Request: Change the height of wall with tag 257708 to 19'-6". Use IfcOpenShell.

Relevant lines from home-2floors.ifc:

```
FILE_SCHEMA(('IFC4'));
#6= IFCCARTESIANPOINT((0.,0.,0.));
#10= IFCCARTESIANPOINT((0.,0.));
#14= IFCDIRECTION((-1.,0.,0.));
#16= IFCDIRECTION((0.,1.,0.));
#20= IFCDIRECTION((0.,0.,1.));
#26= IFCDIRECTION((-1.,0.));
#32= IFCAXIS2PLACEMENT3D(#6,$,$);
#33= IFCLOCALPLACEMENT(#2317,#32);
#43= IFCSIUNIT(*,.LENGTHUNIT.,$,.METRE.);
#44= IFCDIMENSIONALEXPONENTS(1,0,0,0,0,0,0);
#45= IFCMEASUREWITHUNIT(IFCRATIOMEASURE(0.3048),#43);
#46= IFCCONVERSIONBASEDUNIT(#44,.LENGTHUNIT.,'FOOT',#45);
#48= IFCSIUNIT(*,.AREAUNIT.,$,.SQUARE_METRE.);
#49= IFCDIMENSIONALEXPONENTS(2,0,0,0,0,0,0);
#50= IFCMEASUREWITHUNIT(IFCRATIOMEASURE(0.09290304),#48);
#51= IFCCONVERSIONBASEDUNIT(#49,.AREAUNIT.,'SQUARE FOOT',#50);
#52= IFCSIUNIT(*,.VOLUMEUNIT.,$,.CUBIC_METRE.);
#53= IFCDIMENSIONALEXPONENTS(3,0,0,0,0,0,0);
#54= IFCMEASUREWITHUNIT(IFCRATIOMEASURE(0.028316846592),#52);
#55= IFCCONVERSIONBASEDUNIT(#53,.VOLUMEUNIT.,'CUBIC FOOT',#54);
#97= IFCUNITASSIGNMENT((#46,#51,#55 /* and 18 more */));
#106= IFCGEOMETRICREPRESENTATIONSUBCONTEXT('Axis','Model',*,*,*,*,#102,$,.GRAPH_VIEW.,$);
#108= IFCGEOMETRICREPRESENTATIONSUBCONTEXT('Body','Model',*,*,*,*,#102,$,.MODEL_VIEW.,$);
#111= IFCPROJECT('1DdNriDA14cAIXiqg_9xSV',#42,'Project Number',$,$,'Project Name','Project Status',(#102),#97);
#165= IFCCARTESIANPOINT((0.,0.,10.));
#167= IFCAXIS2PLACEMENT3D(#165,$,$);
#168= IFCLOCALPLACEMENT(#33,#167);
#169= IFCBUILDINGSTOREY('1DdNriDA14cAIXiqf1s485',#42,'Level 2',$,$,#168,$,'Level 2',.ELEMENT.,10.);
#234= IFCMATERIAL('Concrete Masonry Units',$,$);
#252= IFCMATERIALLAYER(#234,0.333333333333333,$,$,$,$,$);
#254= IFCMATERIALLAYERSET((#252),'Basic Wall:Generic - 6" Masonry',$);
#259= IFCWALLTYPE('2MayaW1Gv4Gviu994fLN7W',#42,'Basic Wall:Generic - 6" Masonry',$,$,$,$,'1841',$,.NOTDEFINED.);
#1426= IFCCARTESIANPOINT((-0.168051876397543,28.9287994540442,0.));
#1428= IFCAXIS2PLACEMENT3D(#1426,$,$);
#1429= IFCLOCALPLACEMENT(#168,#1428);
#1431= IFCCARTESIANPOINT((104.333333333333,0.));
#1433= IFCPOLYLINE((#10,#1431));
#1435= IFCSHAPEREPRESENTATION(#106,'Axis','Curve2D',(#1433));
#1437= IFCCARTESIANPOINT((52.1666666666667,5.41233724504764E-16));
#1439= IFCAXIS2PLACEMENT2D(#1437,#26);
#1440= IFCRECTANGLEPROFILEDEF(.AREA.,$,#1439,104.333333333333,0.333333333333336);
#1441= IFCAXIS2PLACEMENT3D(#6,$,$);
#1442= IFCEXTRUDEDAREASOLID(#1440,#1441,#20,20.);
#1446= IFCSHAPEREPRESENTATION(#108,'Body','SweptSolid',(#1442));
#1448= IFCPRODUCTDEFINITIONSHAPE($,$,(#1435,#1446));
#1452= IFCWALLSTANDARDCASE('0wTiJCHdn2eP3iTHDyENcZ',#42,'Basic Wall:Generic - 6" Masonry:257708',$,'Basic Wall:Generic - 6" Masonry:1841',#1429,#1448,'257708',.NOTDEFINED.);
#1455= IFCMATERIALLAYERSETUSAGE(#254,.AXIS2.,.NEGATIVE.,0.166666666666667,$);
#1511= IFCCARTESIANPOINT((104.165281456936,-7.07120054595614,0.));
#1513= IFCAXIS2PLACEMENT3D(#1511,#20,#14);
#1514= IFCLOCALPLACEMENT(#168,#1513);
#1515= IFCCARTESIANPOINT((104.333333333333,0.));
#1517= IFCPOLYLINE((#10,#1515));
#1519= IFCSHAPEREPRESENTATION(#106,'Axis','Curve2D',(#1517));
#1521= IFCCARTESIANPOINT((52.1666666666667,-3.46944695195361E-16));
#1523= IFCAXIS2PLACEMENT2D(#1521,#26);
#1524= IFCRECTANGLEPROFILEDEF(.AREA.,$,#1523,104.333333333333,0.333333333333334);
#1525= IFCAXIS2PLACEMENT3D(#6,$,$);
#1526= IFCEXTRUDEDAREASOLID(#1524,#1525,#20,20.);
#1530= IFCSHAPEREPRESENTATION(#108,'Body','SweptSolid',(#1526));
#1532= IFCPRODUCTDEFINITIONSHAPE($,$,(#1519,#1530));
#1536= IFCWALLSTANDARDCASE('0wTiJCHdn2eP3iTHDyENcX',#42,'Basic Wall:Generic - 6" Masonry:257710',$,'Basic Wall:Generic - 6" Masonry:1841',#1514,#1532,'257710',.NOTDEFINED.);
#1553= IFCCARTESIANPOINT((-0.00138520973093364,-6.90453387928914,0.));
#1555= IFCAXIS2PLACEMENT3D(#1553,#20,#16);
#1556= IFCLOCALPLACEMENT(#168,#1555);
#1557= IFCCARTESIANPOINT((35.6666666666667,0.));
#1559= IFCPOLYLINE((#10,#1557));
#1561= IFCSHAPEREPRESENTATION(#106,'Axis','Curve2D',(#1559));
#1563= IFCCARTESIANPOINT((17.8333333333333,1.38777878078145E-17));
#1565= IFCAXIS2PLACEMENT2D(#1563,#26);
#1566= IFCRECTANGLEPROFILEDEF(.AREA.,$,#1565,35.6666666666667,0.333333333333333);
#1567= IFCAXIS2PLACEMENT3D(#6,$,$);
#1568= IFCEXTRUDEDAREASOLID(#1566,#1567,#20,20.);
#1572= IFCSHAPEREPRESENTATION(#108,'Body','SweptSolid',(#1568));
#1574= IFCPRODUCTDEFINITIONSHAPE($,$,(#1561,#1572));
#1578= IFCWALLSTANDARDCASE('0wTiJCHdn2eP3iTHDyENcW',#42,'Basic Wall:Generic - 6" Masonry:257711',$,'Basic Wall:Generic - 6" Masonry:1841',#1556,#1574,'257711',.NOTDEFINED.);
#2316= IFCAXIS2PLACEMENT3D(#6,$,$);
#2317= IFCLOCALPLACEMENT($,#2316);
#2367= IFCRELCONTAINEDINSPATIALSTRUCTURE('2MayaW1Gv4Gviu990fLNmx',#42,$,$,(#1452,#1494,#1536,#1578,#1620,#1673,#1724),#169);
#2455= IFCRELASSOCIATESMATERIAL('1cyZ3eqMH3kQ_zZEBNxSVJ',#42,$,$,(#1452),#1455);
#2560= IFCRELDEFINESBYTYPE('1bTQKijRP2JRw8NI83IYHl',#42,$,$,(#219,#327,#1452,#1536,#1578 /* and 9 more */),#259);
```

```python
import ifcopenshell
import ifcopenshell.geom
import ifcopenshell.util.representation
import ifcopenshell.util.shape
import ifcopenshell.util.unit

model = ifcopenshell.open("home-2floors.ifc")
unit_scale = ifcopenshell.util.unit.calculate_unit_scale(model)
settings = ifcopenshell.geom.settings()


def volume(element):
    """Net volume in cubic metres, openings subtracted."""
    shape = ifcopenshell.geom.create_shape(settings, element)
    return ifcopenshell.util.shape.get_volume(shape.geometry)


wall = model.by_guid("0wTiJCHdn2eP3iTHDyENcZ")
before = volume(wall)

body = ifcopenshell.util.representation.get_representation(wall, "Model", "Body")
solid = body.Items[0]
old_height = solid.Depth
solid.Depth = 234 * 0.0254 / unit_scale
after = volume(wall)

print(f"height {old_height:g} -> {solid.Depth:g}, volume {before:.3f} -> {after:.3f} m3")

model.write("home-2floors_rev.ifc")
```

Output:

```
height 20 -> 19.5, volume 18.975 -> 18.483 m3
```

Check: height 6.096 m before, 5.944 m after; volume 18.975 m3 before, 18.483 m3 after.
